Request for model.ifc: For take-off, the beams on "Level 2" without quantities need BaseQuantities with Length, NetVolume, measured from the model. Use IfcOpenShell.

First a look at what the model holds.

```python
import ifcopenshell
import ifcopenshell.util.element
import ifcopenshell.util.unit

model = ifcopenshell.open("model.ifc")
print(model.schema)
for unit_type in ("LENGTHUNIT", "AREAUNIT", "VOLUMEUNIT"):
    print(unit_type, ifcopenshell.util.unit.calculate_unit_scale(model, unit_type))
storey = next(s for s in model.by_type("IfcBuildingStorey") if s.Name == "Level 2")
beams = [e for e in ifcopenshell.util.element.get_decomposition(storey) if e.is_a("IfcBeam")]
for e in sorted(beams, key=lambda e: e.id()):
    print(e.id(), e.is_a(), e.Name, list(ifcopenshell.util.element.get_psets(e, qtos_only=True)), sep=" | ")
```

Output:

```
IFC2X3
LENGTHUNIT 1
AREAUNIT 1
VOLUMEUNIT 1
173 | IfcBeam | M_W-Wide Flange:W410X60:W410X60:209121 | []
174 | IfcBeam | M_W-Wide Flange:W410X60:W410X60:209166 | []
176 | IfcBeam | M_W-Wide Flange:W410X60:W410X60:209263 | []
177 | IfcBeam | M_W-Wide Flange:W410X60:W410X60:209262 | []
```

```python
import ifcopenshell
import ifcopenshell.api.pset
import ifcopenshell.geom
import ifcopenshell.util.element
import ifcopenshell.util.shape
import ifcopenshell.util.unit

model = ifcopenshell.open("model.ifc")
unit_scale = ifcopenshell.util.unit.calculate_unit_scale(model)
volume_scale = ifcopenshell.util.unit.calculate_unit_scale(model, "VOLUMEUNIT")
settings = ifcopenshell.geom.settings()

storey = next(s for s in model.by_type("IfcBuildingStorey") if s.Name == "Level 2")
beams = [e for e in ifcopenshell.util.element.get_decomposition(storey) if e.is_a("IfcBeam")]

for e in sorted(beams, key=lambda e: e.id()):
    if ifcopenshell.util.element.get_psets(e, qtos_only=True, should_inherit=False):
        continue
    # Geometry comes back in metres, in the element's own axes.
    shape = ifcopenshell.geom.create_shape(settings, e)
    values = {
        "Length": ifcopenshell.util.shape.get_max_xyz(shape.geometry) / unit_scale,
        "NetVolume": ifcopenshell.util.shape.get_volume(shape.geometry) / volume_scale,
    }
    qto = ifcopenshell.api.pset.add_qto(model, product=e, name="BaseQuantities")
    ifcopenshell.api.pset.edit_qto(model, qto=qto, properties=values)
    print(e.id(), {k: round(v, 3) for k, v in values.items()})

model.write("model-out.ifc")
```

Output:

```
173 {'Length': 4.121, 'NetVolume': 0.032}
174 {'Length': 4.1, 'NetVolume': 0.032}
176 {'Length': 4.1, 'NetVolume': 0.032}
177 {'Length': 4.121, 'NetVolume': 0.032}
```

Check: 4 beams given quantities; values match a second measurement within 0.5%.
